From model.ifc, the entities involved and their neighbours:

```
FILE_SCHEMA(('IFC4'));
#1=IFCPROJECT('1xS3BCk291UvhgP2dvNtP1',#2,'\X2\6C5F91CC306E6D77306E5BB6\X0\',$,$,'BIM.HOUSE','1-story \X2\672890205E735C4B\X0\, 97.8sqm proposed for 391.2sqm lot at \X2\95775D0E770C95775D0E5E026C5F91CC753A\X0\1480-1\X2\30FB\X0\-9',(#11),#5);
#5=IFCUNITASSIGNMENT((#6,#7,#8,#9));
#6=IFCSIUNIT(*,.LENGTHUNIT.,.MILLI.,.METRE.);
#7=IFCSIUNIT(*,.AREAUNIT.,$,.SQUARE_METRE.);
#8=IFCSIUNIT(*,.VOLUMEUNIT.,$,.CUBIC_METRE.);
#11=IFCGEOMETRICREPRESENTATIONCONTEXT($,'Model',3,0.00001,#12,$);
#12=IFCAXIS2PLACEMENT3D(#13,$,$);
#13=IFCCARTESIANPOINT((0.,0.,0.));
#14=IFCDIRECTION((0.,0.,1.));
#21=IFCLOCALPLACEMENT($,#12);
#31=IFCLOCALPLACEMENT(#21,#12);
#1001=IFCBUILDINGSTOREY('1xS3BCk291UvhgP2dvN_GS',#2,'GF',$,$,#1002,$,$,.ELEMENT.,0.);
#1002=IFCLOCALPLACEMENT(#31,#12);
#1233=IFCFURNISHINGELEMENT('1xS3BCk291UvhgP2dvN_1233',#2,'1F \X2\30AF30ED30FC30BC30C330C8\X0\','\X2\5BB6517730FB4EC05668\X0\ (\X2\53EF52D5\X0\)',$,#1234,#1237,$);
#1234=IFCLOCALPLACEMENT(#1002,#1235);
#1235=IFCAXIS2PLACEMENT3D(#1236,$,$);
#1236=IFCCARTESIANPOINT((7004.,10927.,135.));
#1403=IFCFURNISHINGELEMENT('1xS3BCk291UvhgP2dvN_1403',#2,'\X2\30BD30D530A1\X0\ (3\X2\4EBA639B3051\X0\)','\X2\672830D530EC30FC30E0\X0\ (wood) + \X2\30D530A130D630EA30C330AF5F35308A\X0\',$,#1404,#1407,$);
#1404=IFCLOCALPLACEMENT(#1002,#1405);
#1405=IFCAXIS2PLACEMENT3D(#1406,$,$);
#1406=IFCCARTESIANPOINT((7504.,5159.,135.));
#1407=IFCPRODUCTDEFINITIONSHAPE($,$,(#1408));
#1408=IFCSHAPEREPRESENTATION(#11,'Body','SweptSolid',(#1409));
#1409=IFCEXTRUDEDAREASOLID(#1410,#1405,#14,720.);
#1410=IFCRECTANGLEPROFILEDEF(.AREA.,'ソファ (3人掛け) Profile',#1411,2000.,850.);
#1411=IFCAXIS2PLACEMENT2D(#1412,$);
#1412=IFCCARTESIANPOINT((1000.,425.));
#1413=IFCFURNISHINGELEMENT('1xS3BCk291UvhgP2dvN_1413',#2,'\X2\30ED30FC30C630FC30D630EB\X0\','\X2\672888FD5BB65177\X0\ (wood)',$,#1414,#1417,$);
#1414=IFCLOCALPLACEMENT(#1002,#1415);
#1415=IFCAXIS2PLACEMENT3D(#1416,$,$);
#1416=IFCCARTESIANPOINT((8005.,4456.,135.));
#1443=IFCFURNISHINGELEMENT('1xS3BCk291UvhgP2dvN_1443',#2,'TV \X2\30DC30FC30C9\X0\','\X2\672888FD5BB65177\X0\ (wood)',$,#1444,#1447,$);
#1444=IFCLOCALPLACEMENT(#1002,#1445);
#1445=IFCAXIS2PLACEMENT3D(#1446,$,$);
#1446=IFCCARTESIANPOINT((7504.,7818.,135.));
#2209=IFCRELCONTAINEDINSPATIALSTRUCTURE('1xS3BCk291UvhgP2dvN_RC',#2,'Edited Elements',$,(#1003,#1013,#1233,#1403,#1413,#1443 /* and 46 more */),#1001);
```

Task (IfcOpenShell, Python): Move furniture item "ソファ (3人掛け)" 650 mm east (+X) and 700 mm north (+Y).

```python
import ifcopenshell
import ifcopenshell.api.geometry
import ifcopenshell.util.placement
import ifcopenshell.util.unit

model = ifcopenshell.open("model.ifc")
unit_scale = ifcopenshell.util.unit.calculate_unit_scale(model)

item = model.by_id(1403)
matrix = ifcopenshell.util.placement.get_local_placement(item.ObjectPlacement)
matrix[0, 3] += 0.65 / unit_scale
matrix[1, 3] += 0.7 / unit_scale
ifcopenshell.api.geometry.edit_object_placement(model, product=item, matrix=matrix, is_si=False)

print(ifcopenshell.util.placement.get_local_placement(item.ObjectPlacement).round(3) + 0.0)

model.write("model_v2.ifc")
```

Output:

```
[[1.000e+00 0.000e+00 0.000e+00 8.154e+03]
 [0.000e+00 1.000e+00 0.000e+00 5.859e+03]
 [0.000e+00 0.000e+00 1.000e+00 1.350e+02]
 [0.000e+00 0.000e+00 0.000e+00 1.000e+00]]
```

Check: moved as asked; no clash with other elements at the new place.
